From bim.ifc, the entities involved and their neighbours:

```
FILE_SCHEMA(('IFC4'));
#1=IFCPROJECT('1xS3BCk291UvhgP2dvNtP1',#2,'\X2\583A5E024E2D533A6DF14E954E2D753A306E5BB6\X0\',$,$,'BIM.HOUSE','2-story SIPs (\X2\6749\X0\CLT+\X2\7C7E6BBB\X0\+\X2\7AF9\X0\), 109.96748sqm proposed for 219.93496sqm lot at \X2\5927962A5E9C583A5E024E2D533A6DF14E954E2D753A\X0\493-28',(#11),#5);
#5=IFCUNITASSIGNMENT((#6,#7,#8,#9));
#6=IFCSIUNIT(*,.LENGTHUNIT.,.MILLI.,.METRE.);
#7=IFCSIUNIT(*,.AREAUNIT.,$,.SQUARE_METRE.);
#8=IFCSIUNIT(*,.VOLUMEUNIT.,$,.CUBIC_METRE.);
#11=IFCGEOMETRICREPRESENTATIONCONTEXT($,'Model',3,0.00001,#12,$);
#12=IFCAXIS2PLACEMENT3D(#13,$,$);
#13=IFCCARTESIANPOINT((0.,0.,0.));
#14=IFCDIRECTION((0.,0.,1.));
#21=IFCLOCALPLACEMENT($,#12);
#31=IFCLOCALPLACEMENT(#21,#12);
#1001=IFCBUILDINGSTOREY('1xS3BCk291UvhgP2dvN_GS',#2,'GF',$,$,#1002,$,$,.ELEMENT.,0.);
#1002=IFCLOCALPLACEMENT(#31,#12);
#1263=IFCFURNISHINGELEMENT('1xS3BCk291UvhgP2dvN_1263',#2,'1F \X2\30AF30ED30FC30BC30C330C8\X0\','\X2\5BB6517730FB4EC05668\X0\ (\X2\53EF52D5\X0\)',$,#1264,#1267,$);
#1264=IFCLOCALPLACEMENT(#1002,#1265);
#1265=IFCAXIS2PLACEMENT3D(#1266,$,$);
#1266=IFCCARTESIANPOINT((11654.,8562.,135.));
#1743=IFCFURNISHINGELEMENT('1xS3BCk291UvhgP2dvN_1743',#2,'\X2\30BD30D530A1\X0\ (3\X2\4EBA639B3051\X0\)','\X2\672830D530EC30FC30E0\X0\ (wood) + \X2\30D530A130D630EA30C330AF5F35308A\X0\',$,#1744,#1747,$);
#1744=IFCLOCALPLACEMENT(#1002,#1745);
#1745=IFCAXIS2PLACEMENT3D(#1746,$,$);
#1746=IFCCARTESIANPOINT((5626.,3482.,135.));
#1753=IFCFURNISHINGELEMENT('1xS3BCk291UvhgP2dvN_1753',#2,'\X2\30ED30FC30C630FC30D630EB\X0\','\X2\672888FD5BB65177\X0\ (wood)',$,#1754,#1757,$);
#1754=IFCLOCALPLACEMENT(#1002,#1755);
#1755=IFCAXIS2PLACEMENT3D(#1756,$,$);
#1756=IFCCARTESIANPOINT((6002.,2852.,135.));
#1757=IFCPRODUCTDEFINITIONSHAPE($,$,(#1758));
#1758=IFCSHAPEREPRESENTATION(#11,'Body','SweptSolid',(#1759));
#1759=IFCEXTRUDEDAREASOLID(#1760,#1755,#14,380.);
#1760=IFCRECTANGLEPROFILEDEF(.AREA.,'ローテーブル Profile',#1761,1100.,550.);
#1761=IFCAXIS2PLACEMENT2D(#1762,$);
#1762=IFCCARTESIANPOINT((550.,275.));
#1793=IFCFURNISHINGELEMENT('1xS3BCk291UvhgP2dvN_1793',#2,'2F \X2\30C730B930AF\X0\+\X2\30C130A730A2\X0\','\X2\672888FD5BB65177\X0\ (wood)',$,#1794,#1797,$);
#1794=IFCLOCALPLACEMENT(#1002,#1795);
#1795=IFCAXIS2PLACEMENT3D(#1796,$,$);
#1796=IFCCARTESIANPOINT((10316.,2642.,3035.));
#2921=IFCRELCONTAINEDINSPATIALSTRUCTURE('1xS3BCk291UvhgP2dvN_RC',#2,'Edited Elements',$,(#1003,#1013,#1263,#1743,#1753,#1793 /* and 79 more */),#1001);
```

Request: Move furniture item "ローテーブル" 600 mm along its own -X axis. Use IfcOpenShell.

```python
import ifcopenshell
import ifcopenshell.api.geometry
import ifcopenshell.util.placement
import ifcopenshell.util.unit

model = ifcopenshell.open("bim.ifc")
unit_scale = ifcopenshell.util.unit.calculate_unit_scale(model)

item = model.by_guid("1xS3BCk291UvhgP2dvN_1753")
matrix = ifcopenshell.util.placement.get_local_placement(item.ObjectPlacement)
matrix[:3, 3] -= matrix[:3, 0] * 0.6 / unit_scale
ifcopenshell.api.geometry.edit_object_placement(model, product=item, matrix=matrix, is_si=False)

print(ifcopenshell.util.placement.get_local_placement(item.ObjectPlacement).round(3) + 0.0)

model.write("bim-out.ifc")
```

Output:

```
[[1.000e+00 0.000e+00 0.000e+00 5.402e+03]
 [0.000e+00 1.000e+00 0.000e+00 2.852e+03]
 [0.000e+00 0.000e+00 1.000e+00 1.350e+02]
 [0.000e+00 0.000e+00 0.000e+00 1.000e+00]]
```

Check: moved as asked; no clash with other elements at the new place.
